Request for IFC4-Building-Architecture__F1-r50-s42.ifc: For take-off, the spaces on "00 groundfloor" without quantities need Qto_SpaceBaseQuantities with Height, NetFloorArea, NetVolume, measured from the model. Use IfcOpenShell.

First a look at what the model holds.

```python
import ifcopenshell
import ifcopenshell.util.element
import ifcopenshell.util.unit

model = ifcopenshell.open("IFC4-Building-Architecture__F1-r50-s42.ifc")
print(model.schema)
for unit_type in ("LENGTHUNIT", "AREAUNIT", "VOLUMEUNIT"):
    print(unit_type, ifcopenshell.util.unit.calculate_unit_scale(model, unit_type))
storey = next(s for s in model.by_type("IfcBuildingStorey") if s.Name == "00 groundfloor")
spaces = [e for e in ifcopenshell.util.element.get_decomposition(storey) if e.is_a("IfcSpace")]
for e in sorted(spaces, key=lambda e: e.id()):
    print(e.id(), e.is_a(), e.Name, list(ifcopenshell.util.element.get_psets(e, qtos_only=True)), sep=" | ")
```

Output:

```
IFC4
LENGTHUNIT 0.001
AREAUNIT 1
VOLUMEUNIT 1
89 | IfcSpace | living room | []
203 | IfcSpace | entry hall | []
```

```python
import ifcopenshell
import ifcopenshell.api.pset
import ifcopenshell.geom
import ifcopenshell.util.element
import ifcopenshell.util.shape
import ifcopenshell.util.unit

model = ifcopenshell.open("IFC4-Building-Architecture__F1-r50-s42.ifc")
unit_scale = ifcopenshell.util.unit.calculate_unit_scale(model)
area_scale = ifcopenshell.util.unit.calculate_unit_scale(model, "AREAUNIT")
volume_scale = ifcopenshell.util.unit.calculate_unit_scale(model, "VOLUMEUNIT")
settings = ifcopenshell.geom.settings()

storey = next(s for s in model.by_type("IfcBuildingStorey") if s.Name == "00 groundfloor")
spaces = [e for e in ifcopenshell.util.element.get_decomposition(storey) if e.is_a("IfcSpace")]

for e in sorted(spaces, key=lambda e: e.id()):
    if ifcopenshell.util.element.get_psets(e, qtos_only=True, should_inherit=False):
        continue
    # Geometry comes back in metres, in the element's own axes.
    shape = ifcopenshell.geom.create_shape(settings, e)
    values = {
        "Height": ifcopenshell.util.shape.get_z(shape.geometry) / unit_scale,
        "NetFloorArea": ifcopenshell.util.shape.get_footprint_area(shape.geometry) / area_scale,
        "NetVolume": ifcopenshell.util.shape.get_volume(shape.geometry) / volume_scale,
    }
    qto = ifcopenshell.api.pset.add_qto(model, product=e, name="Qto_SpaceBaseQuantities")
    ifcopenshell.api.pset.edit_qto(model, qto=qto, properties=values)
    print(e.id(), {k: round(v, 3) for k, v in values.items()})

model.write("IFC4-Building-Architecture__F1-r50-s42_updated.ifc")
```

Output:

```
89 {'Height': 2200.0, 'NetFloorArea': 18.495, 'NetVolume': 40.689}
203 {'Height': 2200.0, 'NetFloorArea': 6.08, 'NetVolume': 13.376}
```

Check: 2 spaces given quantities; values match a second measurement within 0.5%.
